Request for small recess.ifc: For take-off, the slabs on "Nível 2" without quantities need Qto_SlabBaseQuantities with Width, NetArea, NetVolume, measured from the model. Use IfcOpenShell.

First a look at what the model holds.

```python
import ifcopenshell
import ifcopenshell.util.element
import ifcopenshell.util.unit

model = ifcopenshell.open("small recess.ifc")
print(model.schema)
for unit_type in ("LENGTHUNIT", "AREAUNIT", "VOLUMEUNIT"):
    print(unit_type, ifcopenshell.util.unit.calculate_unit_scale(model, unit_type))
storey = next(s for s in model.by_type("IfcBuildingStorey") if s.Name == "Nível 2")
slabs = [e for e in ifcopenshell.util.element.get_decomposition(storey) if e.is_a("IfcSlab")]
for e in sorted(slabs, key=lambda e: e.id()):
    print(e.id(), e.is_a(), e.Name, list(ifcopenshell.util.element.get_psets(e, qtos_only=True)), sep=" | ")
```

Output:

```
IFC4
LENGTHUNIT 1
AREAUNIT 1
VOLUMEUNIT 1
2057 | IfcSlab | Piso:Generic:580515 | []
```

```python
import ifcopenshell
import ifcopenshell.api.pset
import ifcopenshell.geom
import ifcopenshell.util.element
import ifcopenshell.util.shape
import ifcopenshell.util.unit

model = ifcopenshell.open("small recess.ifc")
unit_scale = ifcopenshell.util.unit.calculate_unit_scale(model)
area_scale = ifcopenshell.util.unit.calculate_unit_scale(model, "AREAUNIT")
volume_scale = ifcopenshell.util.unit.calculate_unit_scale(model, "VOLUMEUNIT")
settings = ifcopenshell.geom.settings()

storey = next(s for s in model.by_type("IfcBuildingStorey") if s.Name == "Nível 2")
slabs = [e for e in ifcopenshell.util.element.get_decomposition(storey) if e.is_a("IfcSlab")]

for e in sorted(slabs, key=lambda e: e.id()):
    if ifcopenshell.util.element.get_psets(e, qtos_only=True, should_inherit=False):
        continue
    # Geometry comes back in metres, in the element's own axes.
    shape = ifcopenshell.geom.create_shape(settings, e)
    values = {
        "Width": ifcopenshell.util.shape.get_z(shape.geometry) / unit_scale,
        "NetArea": ifcopenshell.util.shape.get_footprint_area(shape.geometry) / area_scale,
        "NetVolume": ifcopenshell.util.shape.get_volume(shape.geometry) / volume_scale,
    }
    qto = ifcopenshell.api.pset.add_qto(model, product=e, name="Qto_SlabBaseQuantities")
    ifcopenshell.api.pset.edit_qto(model, qto=qto, properties=values)
    print(e.id(), {k: round(v, 3) for k, v in values.items()})

model.write("small recess-out.ifc")
```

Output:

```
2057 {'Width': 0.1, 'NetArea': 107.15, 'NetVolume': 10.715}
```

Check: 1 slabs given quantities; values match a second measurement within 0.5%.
